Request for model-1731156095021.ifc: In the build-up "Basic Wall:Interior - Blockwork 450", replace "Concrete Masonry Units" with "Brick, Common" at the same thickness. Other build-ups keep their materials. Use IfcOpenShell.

First a look at what the model holds.

```python
import ifcopenshell
import ifcopenshell.util.element

model = ifcopenshell.open("model-1731156095021.ifc")
print(model.schema)
for layer_set in model.by_type("IfcMaterialLayerSet"):
    if layer_set.LayerSetName == "Basic Wall:Interior - Blockwork 450":
        for layer in layer_set.MaterialLayers:
            print(layer.id(), layer.Material and layer.Material.Name, layer.LayerThickness, sep=" | ")
        print(len(ifcopenshell.util.element.get_elements_by_material(model, layer_set)), "elements and types use it")
print(sorted(m.Name for m in model.by_type("IfcMaterial") if m.Name)[:60])
```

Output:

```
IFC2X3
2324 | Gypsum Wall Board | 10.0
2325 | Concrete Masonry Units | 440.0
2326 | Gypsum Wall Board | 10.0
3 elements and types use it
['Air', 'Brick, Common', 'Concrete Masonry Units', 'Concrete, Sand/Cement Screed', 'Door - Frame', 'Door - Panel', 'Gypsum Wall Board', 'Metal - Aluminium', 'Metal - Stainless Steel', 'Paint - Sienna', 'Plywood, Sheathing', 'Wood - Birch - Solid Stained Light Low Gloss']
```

```python
import ifcopenshell
import ifcopenshell.api.material

model = ifcopenshell.open("model-1731156095021.ifc")

layer_set = next(s for s in model.by_type("IfcMaterialLayerSet") if s.LayerSetName == "Basic Wall:Interior - Blockwork 450")
layer = next(l for l in layer_set.MaterialLayers if l.Material and l.Material.Name == "Concrete Masonry Units")
material = next(m for m in model.by_type("IfcMaterial") if m.Name == "Brick, Common")

# Point this one layer at the other material; renaming the old one would change it everywhere.
ifcopenshell.api.material.edit_layer(model, layer=layer, attributes={}, material=material)

print([l.Material.Name if l.Material else None for l in layer_set.MaterialLayers])

model.write("model-1731156095021-out.ifc")
```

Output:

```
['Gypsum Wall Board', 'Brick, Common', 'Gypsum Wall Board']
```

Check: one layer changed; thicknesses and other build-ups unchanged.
